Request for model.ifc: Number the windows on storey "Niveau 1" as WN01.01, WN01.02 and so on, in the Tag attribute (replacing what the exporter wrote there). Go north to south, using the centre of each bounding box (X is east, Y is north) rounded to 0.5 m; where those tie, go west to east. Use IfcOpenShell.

First a look at what the model holds.

```python
import ifcopenshell
import ifcopenshell.util.element
import ifcopenshell.util.placement

model = ifcopenshell.open("model.ifc")
print(model.schema)
storey = next(s for s in model.by_type("IfcBuildingStorey") if s.Name == "Niveau 1")
windows = [e for e in ifcopenshell.util.element.get_decomposition(storey) if e.is_a("IfcWindow")]
for e in sorted(windows, key=lambda e: e.id()):
    origin = ifcopenshell.util.placement.get_local_placement(e.ObjectPlacement)[:3, 3]
    print(e.id(), e.Tag, e.Name, origin.round(2) + 0.0, sep=" | ")
```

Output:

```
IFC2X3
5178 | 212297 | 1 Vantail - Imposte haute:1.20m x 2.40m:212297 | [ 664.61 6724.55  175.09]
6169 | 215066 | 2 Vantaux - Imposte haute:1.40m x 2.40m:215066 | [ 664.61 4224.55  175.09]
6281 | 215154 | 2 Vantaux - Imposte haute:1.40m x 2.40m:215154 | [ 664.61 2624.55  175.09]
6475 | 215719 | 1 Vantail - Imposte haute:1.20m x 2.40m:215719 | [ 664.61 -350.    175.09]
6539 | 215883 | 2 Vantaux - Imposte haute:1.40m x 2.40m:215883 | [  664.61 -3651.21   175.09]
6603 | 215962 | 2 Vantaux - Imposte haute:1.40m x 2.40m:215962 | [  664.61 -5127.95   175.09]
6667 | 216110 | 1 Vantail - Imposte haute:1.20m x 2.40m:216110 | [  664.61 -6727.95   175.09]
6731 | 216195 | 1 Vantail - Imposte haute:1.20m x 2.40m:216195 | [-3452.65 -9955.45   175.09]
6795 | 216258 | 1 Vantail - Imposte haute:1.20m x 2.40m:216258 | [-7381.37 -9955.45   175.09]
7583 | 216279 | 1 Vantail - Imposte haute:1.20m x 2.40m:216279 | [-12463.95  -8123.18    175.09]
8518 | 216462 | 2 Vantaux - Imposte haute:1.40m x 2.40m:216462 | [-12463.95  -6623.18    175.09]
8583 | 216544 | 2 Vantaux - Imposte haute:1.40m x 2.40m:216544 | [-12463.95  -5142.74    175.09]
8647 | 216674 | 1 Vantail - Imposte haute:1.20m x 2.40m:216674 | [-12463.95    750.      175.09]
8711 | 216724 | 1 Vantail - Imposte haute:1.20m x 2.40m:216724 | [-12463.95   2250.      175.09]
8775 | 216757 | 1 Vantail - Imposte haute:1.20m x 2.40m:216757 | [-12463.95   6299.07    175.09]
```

```python
import ifcopenshell
import ifcopenshell.geom
import ifcopenshell.util.element
import ifcopenshell.util.shape

model = ifcopenshell.open("model.ifc")
settings = ifcopenshell.geom.settings()
settings.set("use-world-coords", True)


def centre(element):
    shape = ifcopenshell.geom.create_shape(settings, element)
    return ifcopenshell.util.shape.get_bbox_centroid(shape.geometry)


storey = next(s for s in model.by_type("IfcBuildingStorey") if s.Name == "Niveau 1")
windows = [e for e in ifcopenshell.util.element.get_decomposition(storey) if e.is_a("IfcWindow")]

# Insertion points can sit at a corner or the storey origin, so sort by the geometry (in metres).
centres = {e: centre(e) for e in windows}
windows.sort(key=lambda e: (-round(centres[e][1] / 0.5), centres[e][0]))

for i, e in enumerate(windows, start=1):
    number = f"WN01.{i:02d}"
    e.Tag = number
    print(e.id(), number)

model.write("model_v2.ifc")
```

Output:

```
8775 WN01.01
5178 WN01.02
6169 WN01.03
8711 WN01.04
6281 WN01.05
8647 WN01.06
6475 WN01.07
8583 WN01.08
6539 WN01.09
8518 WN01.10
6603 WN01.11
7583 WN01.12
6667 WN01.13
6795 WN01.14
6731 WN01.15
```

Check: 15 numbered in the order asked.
